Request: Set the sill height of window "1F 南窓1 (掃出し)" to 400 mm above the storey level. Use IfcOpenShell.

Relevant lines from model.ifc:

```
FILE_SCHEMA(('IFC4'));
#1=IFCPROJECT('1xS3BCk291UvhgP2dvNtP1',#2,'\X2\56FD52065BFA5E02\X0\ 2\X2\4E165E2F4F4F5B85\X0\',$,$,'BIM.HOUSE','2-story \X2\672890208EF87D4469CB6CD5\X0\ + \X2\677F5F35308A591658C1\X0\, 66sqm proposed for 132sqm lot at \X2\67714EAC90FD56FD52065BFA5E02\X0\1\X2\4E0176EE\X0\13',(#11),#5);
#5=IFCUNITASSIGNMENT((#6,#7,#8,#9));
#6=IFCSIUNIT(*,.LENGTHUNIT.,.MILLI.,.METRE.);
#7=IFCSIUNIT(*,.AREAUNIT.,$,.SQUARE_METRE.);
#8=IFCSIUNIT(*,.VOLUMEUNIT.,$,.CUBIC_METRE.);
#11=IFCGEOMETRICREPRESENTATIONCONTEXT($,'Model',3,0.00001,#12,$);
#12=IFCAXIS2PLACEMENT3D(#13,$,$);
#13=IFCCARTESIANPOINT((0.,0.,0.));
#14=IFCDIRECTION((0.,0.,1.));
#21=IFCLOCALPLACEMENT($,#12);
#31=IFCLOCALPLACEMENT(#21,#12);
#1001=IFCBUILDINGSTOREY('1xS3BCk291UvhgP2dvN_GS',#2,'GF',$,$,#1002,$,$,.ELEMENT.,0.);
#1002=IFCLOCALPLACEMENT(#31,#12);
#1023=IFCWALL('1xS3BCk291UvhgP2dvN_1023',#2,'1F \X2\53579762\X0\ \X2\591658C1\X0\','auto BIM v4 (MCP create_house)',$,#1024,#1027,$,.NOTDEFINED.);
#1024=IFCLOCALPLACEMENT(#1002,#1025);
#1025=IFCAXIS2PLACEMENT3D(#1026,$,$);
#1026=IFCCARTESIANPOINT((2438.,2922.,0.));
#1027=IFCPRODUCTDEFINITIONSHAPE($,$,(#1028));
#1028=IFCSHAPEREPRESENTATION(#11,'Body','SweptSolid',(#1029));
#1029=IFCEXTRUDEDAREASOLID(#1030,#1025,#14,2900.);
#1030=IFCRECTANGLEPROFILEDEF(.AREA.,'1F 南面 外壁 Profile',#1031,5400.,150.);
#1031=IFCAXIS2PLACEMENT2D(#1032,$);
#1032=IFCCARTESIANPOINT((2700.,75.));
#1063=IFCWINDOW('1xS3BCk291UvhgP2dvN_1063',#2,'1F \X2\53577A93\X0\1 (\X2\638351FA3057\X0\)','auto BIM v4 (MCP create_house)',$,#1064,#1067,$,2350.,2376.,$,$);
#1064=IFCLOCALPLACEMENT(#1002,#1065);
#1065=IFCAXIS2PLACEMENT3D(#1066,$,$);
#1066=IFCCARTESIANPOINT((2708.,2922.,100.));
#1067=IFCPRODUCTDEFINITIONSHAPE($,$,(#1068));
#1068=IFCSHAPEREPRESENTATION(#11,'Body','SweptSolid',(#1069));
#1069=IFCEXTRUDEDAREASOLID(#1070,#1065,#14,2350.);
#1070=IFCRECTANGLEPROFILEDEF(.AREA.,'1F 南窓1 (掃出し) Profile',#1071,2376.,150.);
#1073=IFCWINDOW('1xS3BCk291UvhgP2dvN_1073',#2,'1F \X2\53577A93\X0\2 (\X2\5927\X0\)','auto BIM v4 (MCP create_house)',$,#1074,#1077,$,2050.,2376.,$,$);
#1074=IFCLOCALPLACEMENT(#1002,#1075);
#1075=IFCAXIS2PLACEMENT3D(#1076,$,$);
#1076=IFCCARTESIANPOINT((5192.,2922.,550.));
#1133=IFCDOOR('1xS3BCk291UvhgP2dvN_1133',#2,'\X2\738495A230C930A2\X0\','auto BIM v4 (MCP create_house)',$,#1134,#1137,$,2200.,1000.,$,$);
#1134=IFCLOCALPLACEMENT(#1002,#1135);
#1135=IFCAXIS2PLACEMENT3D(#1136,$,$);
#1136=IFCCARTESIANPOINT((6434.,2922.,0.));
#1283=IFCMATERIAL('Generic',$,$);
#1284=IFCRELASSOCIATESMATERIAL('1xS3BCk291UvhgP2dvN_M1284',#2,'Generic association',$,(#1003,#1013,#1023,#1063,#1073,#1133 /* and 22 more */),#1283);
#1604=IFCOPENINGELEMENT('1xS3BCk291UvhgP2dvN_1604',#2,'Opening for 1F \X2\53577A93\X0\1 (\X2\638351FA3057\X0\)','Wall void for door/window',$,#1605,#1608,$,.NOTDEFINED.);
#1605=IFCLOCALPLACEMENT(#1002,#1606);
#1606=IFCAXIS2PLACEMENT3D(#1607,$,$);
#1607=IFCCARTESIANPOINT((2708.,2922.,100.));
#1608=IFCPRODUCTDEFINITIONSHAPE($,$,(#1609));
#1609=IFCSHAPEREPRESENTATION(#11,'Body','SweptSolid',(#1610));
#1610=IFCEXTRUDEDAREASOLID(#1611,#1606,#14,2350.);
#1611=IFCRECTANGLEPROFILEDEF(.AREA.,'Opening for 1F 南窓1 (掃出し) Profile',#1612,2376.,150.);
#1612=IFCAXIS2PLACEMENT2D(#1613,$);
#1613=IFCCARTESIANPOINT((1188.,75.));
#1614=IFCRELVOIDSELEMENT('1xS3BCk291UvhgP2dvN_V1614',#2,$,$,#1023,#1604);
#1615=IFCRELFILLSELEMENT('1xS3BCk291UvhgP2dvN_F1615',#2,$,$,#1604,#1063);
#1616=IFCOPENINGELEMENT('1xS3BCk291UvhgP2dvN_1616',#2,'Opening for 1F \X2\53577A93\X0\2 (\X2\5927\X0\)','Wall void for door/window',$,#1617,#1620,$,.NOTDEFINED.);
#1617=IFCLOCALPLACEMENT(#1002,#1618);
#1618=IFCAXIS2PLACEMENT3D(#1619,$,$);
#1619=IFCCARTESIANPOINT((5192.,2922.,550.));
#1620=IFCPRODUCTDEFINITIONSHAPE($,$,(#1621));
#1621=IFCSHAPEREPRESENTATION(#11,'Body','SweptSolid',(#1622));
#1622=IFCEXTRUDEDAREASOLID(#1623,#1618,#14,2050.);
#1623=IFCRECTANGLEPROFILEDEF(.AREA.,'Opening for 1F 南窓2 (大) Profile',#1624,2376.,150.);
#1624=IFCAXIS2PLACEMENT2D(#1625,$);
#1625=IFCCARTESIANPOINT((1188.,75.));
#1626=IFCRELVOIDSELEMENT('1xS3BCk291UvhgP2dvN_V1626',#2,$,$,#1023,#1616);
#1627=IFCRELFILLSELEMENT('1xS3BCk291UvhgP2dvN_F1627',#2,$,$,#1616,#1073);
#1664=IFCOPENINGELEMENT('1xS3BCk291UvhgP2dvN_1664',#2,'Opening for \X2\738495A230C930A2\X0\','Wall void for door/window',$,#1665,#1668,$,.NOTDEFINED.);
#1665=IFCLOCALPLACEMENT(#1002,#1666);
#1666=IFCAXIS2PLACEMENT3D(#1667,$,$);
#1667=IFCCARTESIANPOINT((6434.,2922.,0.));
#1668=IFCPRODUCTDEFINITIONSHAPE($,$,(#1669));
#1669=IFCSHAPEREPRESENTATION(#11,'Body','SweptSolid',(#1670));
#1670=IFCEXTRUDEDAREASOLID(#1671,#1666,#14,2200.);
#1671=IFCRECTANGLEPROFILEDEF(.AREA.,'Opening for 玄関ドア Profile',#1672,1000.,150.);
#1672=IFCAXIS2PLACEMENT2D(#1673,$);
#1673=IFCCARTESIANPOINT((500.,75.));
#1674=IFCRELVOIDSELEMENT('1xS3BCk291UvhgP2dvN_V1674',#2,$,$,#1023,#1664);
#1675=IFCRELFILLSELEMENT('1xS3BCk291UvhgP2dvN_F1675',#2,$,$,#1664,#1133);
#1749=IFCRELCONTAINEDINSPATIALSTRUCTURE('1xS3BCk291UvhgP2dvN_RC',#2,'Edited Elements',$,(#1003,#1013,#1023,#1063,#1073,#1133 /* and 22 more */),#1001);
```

```python
import numpy as np
import ifcopenshell
import ifcopenshell.api.geometry
import ifcopenshell.geom
import ifcopenshell.util.element
import ifcopenshell.util.placement
import ifcopenshell.util.shape
import ifcopenshell.util.unit

model = ifcopenshell.open("model.ifc")
unit_scale = ifcopenshell.util.unit.calculate_unit_scale(model)

window = model.by_guid("1xS3BCk291UvhgP2dvN_1063")
opening = window.FillsVoids[0].RelatingOpeningElement
storey = ifcopenshell.util.element.get_container(window, ifc_class="IfcBuildingStorey")
level = ifcopenshell.util.placement.get_local_placement(storey.ObjectPlacement)[2, 3]

# The opening's origin need not be at the sill, so measure its lowest point.
shape = ifcopenshell.geom.create_shape(ifcopenshell.geom.settings(), opening)
bottom = ifcopenshell.util.shape.get_shape_bottom_elevation(shape, shape.geometry) / unit_scale
dz = level + 0.4 / unit_scale - bottom

shift = np.array([0.0, 0.0, dz])
# The window is not placed relative to its opening, so move both.
for product in (opening, window):
    matrix = ifcopenshell.util.placement.get_local_placement(product.ObjectPlacement)
    matrix[:3, 3] += shift
    ifcopenshell.api.geometry.edit_object_placement(model, product=product, matrix=matrix, is_si=False)

print(f"moved by {dz * unit_scale:+.3f} m")

model.write("model_edited.ifc")
```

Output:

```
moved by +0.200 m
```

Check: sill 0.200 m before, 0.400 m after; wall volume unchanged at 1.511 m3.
